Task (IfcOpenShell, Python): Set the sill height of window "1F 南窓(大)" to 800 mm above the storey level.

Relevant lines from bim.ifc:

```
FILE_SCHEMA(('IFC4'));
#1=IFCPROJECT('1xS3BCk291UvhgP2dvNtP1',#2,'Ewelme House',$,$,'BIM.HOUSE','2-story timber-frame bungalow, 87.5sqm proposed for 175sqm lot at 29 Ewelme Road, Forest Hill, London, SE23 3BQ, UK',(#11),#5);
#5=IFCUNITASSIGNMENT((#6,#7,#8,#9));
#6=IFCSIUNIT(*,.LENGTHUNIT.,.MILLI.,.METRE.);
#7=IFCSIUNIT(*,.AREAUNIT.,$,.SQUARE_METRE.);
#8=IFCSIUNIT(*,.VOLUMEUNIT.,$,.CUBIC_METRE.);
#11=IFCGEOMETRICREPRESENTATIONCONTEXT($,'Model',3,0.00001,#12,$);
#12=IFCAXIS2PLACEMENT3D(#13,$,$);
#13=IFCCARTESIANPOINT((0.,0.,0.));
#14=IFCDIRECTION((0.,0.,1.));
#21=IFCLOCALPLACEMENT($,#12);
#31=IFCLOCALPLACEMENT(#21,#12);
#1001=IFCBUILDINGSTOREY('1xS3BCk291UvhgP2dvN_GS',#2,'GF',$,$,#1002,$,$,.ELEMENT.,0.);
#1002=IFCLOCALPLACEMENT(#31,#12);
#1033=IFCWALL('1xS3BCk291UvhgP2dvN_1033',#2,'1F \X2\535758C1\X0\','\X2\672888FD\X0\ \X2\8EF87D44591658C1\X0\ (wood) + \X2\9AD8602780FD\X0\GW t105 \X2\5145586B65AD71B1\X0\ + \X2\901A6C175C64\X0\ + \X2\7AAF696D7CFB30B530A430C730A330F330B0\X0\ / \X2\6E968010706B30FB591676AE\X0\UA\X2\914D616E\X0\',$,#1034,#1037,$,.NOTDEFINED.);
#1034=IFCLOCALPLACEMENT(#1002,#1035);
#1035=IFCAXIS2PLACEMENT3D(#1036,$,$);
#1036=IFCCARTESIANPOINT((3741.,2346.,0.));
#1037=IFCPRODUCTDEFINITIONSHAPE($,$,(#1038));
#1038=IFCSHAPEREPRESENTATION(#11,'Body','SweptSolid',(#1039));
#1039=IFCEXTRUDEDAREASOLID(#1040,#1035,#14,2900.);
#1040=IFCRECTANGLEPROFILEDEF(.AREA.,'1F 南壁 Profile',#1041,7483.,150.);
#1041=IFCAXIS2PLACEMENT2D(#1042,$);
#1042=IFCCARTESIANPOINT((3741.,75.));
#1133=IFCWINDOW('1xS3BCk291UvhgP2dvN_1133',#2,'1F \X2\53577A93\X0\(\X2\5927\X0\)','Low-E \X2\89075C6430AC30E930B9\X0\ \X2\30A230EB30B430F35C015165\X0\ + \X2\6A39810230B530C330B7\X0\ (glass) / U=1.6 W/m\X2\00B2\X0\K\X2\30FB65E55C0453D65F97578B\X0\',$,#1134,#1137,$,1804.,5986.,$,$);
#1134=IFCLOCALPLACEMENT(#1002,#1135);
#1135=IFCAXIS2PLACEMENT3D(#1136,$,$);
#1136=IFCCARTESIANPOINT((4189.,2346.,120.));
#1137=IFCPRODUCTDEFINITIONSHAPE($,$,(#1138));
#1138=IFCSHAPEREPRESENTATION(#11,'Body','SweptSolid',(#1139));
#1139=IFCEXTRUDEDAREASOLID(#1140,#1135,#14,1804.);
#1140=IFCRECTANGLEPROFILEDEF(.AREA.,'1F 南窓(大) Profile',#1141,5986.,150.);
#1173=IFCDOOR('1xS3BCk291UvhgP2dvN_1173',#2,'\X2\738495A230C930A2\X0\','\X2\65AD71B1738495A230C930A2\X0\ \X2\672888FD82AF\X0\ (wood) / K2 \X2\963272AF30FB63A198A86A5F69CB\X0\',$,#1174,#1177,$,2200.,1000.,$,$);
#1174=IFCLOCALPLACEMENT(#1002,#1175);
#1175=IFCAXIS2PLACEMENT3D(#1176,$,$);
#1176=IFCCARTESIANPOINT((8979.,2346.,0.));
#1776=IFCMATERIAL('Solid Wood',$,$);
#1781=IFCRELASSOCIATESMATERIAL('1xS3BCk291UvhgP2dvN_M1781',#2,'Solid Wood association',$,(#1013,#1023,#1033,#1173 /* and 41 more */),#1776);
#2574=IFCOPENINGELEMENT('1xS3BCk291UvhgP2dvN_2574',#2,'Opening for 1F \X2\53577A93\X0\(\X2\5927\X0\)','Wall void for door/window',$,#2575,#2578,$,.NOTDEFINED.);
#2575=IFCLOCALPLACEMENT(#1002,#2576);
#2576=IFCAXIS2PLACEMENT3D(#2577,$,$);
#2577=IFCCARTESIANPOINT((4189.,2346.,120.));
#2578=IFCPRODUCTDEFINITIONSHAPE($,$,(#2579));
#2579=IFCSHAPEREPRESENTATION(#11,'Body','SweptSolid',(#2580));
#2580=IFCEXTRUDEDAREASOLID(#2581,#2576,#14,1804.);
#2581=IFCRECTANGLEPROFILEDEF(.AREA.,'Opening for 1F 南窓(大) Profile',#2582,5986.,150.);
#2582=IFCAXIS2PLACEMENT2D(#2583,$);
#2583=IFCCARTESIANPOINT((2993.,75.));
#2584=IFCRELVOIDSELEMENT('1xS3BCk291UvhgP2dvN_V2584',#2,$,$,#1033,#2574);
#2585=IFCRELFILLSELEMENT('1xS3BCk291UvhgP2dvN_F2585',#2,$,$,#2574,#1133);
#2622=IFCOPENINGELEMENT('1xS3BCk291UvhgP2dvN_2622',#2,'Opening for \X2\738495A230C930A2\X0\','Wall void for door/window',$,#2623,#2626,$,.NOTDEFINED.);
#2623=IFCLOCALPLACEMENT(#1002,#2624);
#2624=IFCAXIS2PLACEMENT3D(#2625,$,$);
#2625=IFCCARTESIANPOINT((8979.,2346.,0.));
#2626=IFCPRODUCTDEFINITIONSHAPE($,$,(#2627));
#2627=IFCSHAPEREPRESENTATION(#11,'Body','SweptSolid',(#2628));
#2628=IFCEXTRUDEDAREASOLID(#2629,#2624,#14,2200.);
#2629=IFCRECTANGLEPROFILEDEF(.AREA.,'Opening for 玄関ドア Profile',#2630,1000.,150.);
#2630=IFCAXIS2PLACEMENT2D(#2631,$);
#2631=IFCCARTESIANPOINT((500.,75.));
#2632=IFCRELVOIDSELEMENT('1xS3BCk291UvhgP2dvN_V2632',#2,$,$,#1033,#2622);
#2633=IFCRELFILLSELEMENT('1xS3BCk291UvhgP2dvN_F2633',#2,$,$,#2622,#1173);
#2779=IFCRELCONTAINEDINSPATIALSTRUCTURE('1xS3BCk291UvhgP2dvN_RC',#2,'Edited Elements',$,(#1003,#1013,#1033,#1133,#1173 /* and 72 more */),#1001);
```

```python
import numpy as np
import ifcopenshell
import ifcopenshell.api.geometry
import ifcopenshell.geom
import ifcopenshell.util.element
import ifcopenshell.util.placement
import ifcopenshell.util.shape
import ifcopenshell.util.unit

model = ifcopenshell.open("bim.ifc")
unit_scale = ifcopenshell.util.unit.calculate_unit_scale(model)

window = model.by_guid("1xS3BCk291UvhgP2dvN_1133")
opening = window.FillsVoids[0].RelatingOpeningElement
storey = ifcopenshell.util.element.get_container(window, ifc_class="IfcBuildingStorey")
level = ifcopenshell.util.placement.get_local_placement(storey.ObjectPlacement)[2, 3]

# The opening's origin need not be at the sill, so measure its lowest point.
shape = ifcopenshell.geom.create_shape(ifcopenshell.geom.settings(), opening)
bottom = ifcopenshell.util.shape.get_shape_bottom_elevation(shape, shape.geometry) / unit_scale
dz = level + 800.0 - bottom

shift = np.array([0.0, 0.0, dz])
# The window is not placed relative to its opening, so move both.
for product in (opening, window):
    matrix = ifcopenshell.util.placement.get_local_placement(product.ObjectPlacement)
    matrix[:3, 3] += shift
    ifcopenshell.api.geometry.edit_object_placement(model, product=product, matrix=matrix, is_si=False)

print(f"moved by {dz * unit_scale:+.3f} m")

model.write("bim_updated.ifc")
```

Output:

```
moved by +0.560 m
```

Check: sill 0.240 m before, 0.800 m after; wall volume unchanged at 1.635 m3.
